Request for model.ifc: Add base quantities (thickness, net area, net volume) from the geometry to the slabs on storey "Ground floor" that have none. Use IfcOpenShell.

First a look at what the model holds.

```python
import ifcopenshell
import ifcopenshell.util.element
import ifcopenshell.util.unit

model = ifcopenshell.open("model.ifc")
print(model.schema)
for unit_type in ("LENGTHUNIT", "AREAUNIT", "VOLUMEUNIT"):
    print(unit_type, ifcopenshell.util.unit.calculate_unit_scale(model, unit_type))
storey = next(s for s in model.by_type("IfcBuildingStorey") if s.Name == "Ground floor")
slabs = [e for e in ifcopenshell.util.element.get_decomposition(storey) if e.is_a("IfcSlab")]
for e in sorted(slabs, key=lambda e: e.id()):
    print(e.id(), e.is_a(), e.Name, list(ifcopenshell.util.element.get_psets(e, qtos_only=True)), sep=" | ")
```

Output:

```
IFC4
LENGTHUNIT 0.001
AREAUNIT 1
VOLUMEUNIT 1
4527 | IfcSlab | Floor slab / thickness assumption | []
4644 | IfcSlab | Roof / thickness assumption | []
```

```python
import ifcopenshell
import ifcopenshell.api.pset
import ifcopenshell.geom
import ifcopenshell.util.element
import ifcopenshell.util.shape
import ifcopenshell.util.unit

model = ifcopenshell.open("model.ifc")
unit_scale = ifcopenshell.util.unit.calculate_unit_scale(model)
area_scale = ifcopenshell.util.unit.calculate_unit_scale(model, "AREAUNIT")
volume_scale = ifcopenshell.util.unit.calculate_unit_scale(model, "VOLUMEUNIT")
settings = ifcopenshell.geom.settings()

storey = next(s for s in model.by_type("IfcBuildingStorey") if s.Name == "Ground floor")
slabs = [e for e in ifcopenshell.util.element.get_decomposition(storey) if e.is_a("IfcSlab")]

for e in sorted(slabs, key=lambda e: e.id()):
    if ifcopenshell.util.element.get_psets(e, qtos_only=True, should_inherit=False):
        continue
    # Geometry comes back in metres, in the element's own axes.
    shape = ifcopenshell.geom.create_shape(settings, e)
    values = {
        "Width": ifcopenshell.util.shape.get_z(shape.geometry) / unit_scale,
        "NetArea": ifcopenshell.util.shape.get_footprint_area(shape.geometry) / area_scale,
        "NetVolume": ifcopenshell.util.shape.get_volume(shape.geometry) / volume_scale,
    }
    qto = ifcopenshell.api.pset.add_qto(model, product=e, name="Qto_SlabBaseQuantities")
    ifcopenshell.api.pset.edit_qto(model, qto=qto, properties=values)
    print(e.id(), {k: round(v, 3) for k, v in values.items()})

model.write("model_edited.ifc")
```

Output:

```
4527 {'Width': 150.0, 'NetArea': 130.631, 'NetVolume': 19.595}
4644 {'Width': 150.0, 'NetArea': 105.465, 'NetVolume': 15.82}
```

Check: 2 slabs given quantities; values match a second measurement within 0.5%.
